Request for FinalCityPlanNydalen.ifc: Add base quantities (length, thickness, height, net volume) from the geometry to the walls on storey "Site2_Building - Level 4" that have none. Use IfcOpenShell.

First a look at what the model holds.

```python
import ifcopenshell
import ifcopenshell.util.element
import ifcopenshell.util.unit

model = ifcopenshell.open("FinalCityPlanNydalen.ifc")
print(model.schema)
for unit_type in ("LENGTHUNIT", "AREAUNIT", "VOLUMEUNIT"):
    print(unit_type, ifcopenshell.util.unit.calculate_unit_scale(model, unit_type))
storey = next(s for s in model.by_type("IfcBuildingStorey") if s.Name == "Site2_Building - Level 4")
walls = [e for e in ifcopenshell.util.element.get_decomposition(storey) if e.is_a("IfcWall")]
for e in sorted(walls, key=lambda e: e.id()):
    print(e.id(), e.is_a(), e.Name, list(ifcopenshell.util.element.get_psets(e, qtos_only=True)), sep=" | ")
```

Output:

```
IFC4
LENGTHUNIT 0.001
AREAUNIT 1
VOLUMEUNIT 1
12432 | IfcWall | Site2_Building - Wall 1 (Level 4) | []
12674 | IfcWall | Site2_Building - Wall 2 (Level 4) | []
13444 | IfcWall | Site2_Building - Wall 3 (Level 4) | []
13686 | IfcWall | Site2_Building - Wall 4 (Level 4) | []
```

```python
import ifcopenshell
import ifcopenshell.api.pset
import ifcopenshell.geom
import ifcopenshell.util.element
import ifcopenshell.util.shape
import ifcopenshell.util.unit

model = ifcopenshell.open("FinalCityPlanNydalen.ifc")
unit_scale = ifcopenshell.util.unit.calculate_unit_scale(model)
volume_scale = ifcopenshell.util.unit.calculate_unit_scale(model, "VOLUMEUNIT")
settings = ifcopenshell.geom.settings()

storey = next(s for s in model.by_type("IfcBuildingStorey") if s.Name == "Site2_Building - Level 4")
walls = [e for e in ifcopenshell.util.element.get_decomposition(storey) if e.is_a("IfcWall")]

for e in sorted(walls, key=lambda e: e.id()):
    if ifcopenshell.util.element.get_psets(e, qtos_only=True, should_inherit=False):
        continue
    # Geometry comes back in metres, in the element's own axes.
    shape = ifcopenshell.geom.create_shape(settings, e)
    values = {
        "Length": ifcopenshell.util.shape.get_x(shape.geometry) / unit_scale,
        "Width": ifcopenshell.util.shape.get_y(shape.geometry) / unit_scale,
        "Height": ifcopenshell.util.shape.get_z(shape.geometry) / unit_scale,
        "NetVolume": ifcopenshell.util.shape.get_volume(shape.geometry) / volume_scale,
    }
    qto = ifcopenshell.api.pset.add_qto(model, product=e, name="Qto_WallBaseQuantities")
    ifcopenshell.api.pset.edit_qto(model, qto=qto, properties=values)
    print(e.id(), {k: round(v, 3) for k, v in values.items()})

model.write("FinalCityPlanNydalen_updated.ifc")
```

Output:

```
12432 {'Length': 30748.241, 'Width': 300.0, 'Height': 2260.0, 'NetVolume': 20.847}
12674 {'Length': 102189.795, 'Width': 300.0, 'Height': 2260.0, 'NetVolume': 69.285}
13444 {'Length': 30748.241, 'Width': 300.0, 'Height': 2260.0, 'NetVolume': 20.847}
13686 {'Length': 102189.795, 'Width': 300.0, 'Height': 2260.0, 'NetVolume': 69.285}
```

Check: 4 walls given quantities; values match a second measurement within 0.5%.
